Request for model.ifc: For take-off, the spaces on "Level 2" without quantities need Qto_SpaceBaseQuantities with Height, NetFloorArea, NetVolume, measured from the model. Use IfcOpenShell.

First a look at what the model holds.

```python
import ifcopenshell
import ifcopenshell.util.element
import ifcopenshell.util.unit

model = ifcopenshell.open("model.ifc")
print(model.schema)
for unit_type in ("LENGTHUNIT", "AREAUNIT", "VOLUMEUNIT"):
    print(unit_type, ifcopenshell.util.unit.calculate_unit_scale(model, unit_type))
storey = next(s for s in model.by_type("IfcBuildingStorey") if s.Name == "Level 2")
spaces = [e for e in ifcopenshell.util.element.get_decomposition(storey) if e.is_a("IfcSpace")]
for e in sorted(spaces, key=lambda e: e.id()):
    print(e.id(), e.is_a(), e.Name, list(ifcopenshell.util.element.get_psets(e, qtos_only=True)), sep=" | ")
```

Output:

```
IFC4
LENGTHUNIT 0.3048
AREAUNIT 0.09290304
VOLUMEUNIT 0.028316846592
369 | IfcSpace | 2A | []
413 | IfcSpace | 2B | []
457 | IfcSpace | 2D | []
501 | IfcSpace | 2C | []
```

```python
import ifcopenshell
import ifcopenshell.api.pset
import ifcopenshell.geom
import ifcopenshell.util.element
import ifcopenshell.util.shape
import ifcopenshell.util.unit

model = ifcopenshell.open("model.ifc")
unit_scale = ifcopenshell.util.unit.calculate_unit_scale(model)
area_scale = ifcopenshell.util.unit.calculate_unit_scale(model, "AREAUNIT")
volume_scale = ifcopenshell.util.unit.calculate_unit_scale(model, "VOLUMEUNIT")
settings = ifcopenshell.geom.settings()

storey = next(s for s in model.by_type("IfcBuildingStorey") if s.Name == "Level 2")
spaces = [e for e in ifcopenshell.util.element.get_decomposition(storey) if e.is_a("IfcSpace")]

for e in sorted(spaces, key=lambda e: e.id()):
    if ifcopenshell.util.element.get_psets(e, qtos_only=True, should_inherit=False):
        continue
    # Geometry comes back in metres, in the element's own axes.
    shape = ifcopenshell.geom.create_shape(settings, e)
    values = {
        "Height": ifcopenshell.util.shape.get_z(shape.geometry) / unit_scale,
        "NetFloorArea": ifcopenshell.util.shape.get_footprint_area(shape.geometry) / area_scale,
        "NetVolume": ifcopenshell.util.shape.get_volume(shape.geometry) / volume_scale,
    }
    qto = ifcopenshell.api.pset.add_qto(model, product=e, name="Qto_SpaceBaseQuantities")
    ifcopenshell.api.pset.edit_qto(model, qto=qto, properties=values)
    print(e.id(), {k: round(v, 3) for k, v in values.items()})

model.write("model_v2.ifc")
```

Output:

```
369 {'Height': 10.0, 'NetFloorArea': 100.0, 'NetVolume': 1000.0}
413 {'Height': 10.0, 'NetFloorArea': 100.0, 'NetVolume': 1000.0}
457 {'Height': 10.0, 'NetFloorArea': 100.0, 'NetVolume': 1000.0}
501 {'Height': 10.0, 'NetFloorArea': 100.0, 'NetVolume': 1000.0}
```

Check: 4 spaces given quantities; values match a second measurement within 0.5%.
